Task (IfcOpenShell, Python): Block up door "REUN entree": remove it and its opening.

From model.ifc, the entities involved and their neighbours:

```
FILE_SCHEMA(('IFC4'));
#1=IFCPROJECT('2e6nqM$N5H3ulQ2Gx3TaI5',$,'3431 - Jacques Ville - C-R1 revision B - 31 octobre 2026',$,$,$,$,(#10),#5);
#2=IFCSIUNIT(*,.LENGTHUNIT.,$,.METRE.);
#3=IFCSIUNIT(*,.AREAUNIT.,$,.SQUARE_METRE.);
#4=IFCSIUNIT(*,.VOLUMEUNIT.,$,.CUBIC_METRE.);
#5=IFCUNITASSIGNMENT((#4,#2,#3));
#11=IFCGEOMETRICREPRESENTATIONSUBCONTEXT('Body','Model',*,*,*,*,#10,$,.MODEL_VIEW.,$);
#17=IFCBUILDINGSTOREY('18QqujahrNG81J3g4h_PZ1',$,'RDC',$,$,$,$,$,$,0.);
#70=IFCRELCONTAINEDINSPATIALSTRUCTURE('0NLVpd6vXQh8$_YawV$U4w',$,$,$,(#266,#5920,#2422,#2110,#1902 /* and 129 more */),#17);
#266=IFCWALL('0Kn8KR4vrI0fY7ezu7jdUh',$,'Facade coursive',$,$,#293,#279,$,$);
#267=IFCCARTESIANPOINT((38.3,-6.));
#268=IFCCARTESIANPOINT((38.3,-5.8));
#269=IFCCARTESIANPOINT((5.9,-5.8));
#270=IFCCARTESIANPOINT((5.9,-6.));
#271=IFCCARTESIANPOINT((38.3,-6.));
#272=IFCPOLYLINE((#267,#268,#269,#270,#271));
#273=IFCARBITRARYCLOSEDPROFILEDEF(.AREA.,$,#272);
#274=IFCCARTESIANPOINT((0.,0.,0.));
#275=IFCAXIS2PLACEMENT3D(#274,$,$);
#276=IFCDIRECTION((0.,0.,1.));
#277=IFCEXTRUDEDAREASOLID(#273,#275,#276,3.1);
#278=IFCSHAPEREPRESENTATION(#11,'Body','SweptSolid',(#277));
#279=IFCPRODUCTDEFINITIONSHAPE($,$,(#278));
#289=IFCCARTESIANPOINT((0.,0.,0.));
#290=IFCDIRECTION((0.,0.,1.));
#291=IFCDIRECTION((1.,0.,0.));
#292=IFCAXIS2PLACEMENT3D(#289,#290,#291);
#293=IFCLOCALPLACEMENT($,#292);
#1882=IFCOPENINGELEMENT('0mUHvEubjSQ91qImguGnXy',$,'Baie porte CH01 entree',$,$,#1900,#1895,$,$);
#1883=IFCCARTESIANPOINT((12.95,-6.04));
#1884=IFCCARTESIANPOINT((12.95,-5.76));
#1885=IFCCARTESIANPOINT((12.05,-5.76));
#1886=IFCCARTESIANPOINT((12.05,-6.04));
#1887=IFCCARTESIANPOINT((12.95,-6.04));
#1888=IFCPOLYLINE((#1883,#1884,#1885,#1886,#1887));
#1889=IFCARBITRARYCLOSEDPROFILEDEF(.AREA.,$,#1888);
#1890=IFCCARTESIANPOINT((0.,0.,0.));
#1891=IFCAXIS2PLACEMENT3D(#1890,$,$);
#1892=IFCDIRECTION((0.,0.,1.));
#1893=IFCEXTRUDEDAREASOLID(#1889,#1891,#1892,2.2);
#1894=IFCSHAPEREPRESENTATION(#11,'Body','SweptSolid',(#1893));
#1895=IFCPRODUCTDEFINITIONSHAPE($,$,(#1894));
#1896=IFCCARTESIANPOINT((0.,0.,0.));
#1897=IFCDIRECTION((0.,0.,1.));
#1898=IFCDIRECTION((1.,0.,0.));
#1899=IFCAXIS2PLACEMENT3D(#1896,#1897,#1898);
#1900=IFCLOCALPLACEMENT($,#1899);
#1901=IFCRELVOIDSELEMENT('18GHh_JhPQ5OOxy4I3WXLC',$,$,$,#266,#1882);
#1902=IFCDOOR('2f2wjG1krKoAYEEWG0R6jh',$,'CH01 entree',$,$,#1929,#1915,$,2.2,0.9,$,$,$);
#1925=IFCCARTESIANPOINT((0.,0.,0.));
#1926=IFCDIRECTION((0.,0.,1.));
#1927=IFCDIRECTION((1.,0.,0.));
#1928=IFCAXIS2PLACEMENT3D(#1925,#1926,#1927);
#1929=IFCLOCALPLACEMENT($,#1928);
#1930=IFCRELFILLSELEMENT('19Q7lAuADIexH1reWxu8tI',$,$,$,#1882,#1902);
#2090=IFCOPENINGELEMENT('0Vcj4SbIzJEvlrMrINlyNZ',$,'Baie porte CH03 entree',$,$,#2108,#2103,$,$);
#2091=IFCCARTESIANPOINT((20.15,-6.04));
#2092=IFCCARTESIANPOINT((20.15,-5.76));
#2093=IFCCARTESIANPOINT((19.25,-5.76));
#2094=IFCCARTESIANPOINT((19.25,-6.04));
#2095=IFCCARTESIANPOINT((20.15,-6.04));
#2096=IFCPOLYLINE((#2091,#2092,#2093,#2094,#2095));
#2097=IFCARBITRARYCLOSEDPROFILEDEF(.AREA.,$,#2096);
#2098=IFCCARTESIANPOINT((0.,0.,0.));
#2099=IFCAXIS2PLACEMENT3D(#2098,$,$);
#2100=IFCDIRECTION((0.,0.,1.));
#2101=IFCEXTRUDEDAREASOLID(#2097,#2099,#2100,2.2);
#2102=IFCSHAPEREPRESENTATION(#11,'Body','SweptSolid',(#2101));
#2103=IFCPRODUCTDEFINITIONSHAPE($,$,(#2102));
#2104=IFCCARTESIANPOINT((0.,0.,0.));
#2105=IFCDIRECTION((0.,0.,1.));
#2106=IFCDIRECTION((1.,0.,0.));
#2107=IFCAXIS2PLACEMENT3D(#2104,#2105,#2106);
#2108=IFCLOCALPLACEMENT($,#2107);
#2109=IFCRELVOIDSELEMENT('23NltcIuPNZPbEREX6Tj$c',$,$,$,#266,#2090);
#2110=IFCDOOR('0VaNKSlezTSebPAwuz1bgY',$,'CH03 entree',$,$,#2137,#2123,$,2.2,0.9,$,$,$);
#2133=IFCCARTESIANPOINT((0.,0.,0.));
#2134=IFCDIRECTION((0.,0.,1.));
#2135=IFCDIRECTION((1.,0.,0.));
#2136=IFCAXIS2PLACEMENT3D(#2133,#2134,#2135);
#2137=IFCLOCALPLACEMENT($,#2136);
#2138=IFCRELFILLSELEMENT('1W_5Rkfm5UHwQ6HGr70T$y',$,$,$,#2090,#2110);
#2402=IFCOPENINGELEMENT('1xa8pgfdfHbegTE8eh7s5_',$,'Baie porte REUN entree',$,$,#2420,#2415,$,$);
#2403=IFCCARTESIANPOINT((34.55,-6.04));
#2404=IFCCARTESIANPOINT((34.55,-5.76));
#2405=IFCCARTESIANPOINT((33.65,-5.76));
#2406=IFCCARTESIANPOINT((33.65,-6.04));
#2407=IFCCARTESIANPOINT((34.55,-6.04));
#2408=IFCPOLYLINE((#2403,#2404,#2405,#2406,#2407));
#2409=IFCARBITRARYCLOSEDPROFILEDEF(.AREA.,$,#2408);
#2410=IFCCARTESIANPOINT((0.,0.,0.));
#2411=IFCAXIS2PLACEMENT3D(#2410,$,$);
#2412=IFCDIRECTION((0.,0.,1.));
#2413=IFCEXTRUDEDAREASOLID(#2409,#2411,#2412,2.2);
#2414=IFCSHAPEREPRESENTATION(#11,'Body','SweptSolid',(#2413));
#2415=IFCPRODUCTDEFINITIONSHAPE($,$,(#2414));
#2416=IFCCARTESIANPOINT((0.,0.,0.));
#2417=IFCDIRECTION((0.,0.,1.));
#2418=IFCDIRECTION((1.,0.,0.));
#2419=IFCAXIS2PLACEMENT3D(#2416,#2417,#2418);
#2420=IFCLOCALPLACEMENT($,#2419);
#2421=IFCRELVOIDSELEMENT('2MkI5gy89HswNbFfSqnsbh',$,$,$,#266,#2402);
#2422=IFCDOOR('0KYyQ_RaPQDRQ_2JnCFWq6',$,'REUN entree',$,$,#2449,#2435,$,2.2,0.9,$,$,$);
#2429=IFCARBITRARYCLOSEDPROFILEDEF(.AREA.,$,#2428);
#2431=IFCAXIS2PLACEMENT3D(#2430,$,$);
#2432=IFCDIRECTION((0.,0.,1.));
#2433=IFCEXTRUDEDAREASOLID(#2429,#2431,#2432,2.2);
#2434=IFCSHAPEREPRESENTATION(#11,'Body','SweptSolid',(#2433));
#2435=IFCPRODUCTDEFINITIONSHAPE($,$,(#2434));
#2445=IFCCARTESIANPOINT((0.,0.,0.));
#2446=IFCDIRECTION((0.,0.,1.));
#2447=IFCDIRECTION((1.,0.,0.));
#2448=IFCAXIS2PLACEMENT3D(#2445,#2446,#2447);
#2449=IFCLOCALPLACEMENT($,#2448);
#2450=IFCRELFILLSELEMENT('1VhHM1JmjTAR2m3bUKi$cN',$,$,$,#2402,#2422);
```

```python
import ifcopenshell
import ifcopenshell.api.feature
import ifcopenshell.api.root
import ifcopenshell.geom
import ifcopenshell.util.shape

model = ifcopenshell.open("model.ifc")
settings = ifcopenshell.geom.settings()


def volume(element):
    """Net volume in cubic metres, openings subtracted."""
    shape = ifcopenshell.geom.create_shape(settings, element)
    return ifcopenshell.util.shape.get_volume(shape.geometry)


door = model.by_guid("0KYyQ_RaPQDRQ_2JnCFWq6")
opening = door.FillsVoids[0].RelatingOpeningElement
wall = opening.VoidsElements[0].RelatingBuildingElement
before = volume(wall)

ifcopenshell.api.root.remove_product(model, product=door)
ifcopenshell.api.feature.remove_feature(model, feature=opening)

after = volume(wall)

print(f"wall volume {before:.3f} -> {after:.3f} m3")

model.write("model-out.ifc")
```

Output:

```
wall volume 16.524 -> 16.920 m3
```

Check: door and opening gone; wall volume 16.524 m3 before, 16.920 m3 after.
